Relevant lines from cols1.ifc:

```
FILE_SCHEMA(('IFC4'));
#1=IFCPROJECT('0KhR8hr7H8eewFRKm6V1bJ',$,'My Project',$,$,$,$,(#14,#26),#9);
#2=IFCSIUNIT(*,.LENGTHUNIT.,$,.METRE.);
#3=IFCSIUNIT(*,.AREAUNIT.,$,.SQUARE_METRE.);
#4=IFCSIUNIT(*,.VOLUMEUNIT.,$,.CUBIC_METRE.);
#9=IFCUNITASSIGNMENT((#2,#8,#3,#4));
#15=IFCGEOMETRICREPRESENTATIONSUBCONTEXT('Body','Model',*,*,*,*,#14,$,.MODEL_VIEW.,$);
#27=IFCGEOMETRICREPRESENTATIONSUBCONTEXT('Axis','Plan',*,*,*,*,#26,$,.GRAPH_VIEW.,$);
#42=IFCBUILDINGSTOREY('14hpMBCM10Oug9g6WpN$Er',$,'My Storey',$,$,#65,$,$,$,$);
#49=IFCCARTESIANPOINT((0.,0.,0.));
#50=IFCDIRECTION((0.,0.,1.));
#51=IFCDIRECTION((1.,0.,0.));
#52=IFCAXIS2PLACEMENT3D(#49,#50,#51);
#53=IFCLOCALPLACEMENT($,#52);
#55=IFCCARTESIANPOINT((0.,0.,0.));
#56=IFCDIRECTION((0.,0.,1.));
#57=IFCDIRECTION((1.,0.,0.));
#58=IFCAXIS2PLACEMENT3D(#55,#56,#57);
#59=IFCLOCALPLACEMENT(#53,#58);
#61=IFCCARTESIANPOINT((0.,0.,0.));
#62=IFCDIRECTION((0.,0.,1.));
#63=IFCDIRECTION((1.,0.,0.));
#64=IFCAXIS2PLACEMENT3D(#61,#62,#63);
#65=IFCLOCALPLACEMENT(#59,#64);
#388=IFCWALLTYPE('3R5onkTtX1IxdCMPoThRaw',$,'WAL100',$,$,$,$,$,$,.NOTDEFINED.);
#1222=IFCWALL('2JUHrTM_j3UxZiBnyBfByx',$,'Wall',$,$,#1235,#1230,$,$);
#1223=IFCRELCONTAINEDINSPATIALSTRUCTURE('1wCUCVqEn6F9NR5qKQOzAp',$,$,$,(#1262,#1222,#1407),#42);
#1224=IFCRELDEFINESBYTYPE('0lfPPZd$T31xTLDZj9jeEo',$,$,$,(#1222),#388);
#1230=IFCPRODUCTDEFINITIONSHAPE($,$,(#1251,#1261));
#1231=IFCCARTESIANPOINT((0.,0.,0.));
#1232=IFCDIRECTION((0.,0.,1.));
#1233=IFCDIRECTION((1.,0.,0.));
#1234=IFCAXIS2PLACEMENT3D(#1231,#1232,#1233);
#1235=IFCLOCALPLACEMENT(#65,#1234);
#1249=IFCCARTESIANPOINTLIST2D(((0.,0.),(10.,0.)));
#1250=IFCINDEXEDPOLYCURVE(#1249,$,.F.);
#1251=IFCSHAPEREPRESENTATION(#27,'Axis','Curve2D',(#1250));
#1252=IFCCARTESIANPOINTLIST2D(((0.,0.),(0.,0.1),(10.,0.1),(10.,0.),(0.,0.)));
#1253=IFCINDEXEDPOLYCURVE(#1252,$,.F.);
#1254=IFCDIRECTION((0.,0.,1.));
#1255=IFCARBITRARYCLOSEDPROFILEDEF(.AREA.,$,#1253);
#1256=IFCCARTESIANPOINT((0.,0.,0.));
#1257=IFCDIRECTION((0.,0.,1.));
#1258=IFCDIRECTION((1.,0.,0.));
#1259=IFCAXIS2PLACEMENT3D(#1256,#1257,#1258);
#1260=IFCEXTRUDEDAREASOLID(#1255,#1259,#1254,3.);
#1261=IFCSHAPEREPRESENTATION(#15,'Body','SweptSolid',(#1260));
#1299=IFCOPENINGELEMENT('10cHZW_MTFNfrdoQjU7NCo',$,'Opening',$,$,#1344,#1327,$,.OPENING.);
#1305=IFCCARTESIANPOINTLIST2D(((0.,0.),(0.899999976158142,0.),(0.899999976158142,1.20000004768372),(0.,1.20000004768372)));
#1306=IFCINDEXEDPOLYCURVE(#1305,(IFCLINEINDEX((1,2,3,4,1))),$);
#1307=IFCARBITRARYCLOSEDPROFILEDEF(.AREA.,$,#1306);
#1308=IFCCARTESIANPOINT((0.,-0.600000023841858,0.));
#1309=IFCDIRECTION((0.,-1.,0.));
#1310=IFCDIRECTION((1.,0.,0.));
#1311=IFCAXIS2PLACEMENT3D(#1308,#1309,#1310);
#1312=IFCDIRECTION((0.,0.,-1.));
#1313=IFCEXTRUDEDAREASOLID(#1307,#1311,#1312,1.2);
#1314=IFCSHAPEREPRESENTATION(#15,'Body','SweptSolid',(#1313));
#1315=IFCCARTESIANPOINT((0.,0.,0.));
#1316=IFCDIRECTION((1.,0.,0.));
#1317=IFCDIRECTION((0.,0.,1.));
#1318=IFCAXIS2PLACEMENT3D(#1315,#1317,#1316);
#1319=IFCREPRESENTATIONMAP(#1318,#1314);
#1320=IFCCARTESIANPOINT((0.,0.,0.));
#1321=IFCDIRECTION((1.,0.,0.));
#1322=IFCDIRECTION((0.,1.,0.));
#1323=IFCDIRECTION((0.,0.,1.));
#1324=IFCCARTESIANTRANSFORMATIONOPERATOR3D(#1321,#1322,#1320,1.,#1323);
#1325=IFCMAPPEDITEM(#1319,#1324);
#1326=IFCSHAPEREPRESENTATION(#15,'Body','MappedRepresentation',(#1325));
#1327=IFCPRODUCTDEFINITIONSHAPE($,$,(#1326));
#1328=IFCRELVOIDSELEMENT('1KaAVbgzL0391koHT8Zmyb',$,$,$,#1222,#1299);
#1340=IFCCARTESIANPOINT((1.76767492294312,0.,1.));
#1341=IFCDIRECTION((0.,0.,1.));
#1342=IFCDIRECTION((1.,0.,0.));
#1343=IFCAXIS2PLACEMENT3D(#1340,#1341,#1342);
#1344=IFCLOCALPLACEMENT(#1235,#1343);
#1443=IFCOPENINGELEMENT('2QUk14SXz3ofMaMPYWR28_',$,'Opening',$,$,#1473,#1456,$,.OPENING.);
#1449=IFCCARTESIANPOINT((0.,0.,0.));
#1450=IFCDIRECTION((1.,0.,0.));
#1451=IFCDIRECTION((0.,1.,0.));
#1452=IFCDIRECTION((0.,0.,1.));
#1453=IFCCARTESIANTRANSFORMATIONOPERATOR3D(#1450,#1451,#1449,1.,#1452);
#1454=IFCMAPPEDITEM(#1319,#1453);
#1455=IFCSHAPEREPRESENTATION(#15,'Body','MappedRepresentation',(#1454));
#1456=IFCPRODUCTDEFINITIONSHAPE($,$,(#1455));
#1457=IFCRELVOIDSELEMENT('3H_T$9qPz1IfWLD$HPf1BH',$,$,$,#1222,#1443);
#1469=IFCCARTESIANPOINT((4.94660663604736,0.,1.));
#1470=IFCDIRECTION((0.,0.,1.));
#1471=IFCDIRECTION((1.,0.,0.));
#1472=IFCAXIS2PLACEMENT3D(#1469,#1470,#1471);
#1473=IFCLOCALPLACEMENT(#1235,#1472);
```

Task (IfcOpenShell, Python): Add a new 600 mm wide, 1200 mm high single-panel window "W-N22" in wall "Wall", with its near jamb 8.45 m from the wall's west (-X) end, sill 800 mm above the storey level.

```python
import numpy as np
import ifcopenshell
import ifcopenshell.api.feature
import ifcopenshell.api.geometry
import ifcopenshell.api.root
import ifcopenshell.api.spatial
import ifcopenshell.geom
import ifcopenshell.util.element
import ifcopenshell.util.placement
import ifcopenshell.util.representation
import ifcopenshell.util.shape
import ifcopenshell.util.unit

model = ifcopenshell.open("cols1.ifc")
unit_scale = ifcopenshell.util.unit.calculate_unit_scale(model)
settings = ifcopenshell.geom.settings()


def volume(element):
    """Net volume in cubic metres, openings subtracted."""
    shape = ifcopenshell.geom.create_shape(settings, element)
    return ifcopenshell.util.shape.get_volume(shape.geometry)


wall = model.by_guid("2JUHrTM_j3UxZiBnyBfByx")
storey = ifcopenshell.util.element.get_container(wall, ifc_class="IfcBuildingStorey")
context = ifcopenshell.util.representation.get_context(model, "Model", "Body", "MODEL_VIEW")
before = volume(wall)

width, height, from_end, sill = 0.6, 1.2, 8.45, 0.8  # metres

# The wall runs along its own X axis, and the end named is its -X end.
wall_shape = ifcopenshell.geom.create_shape(settings, wall)
x, y, z = ifcopenshell.util.shape.get_vertices(wall_shape.geometry).T
start = x.min() + from_end
face, thickness = float(y.min()), float(y.max() - y.min())
wall_matrix = ifcopenshell.util.placement.get_local_placement(wall.ObjectPlacement)
level = ifcopenshell.util.placement.get_local_placement(storey.ObjectPlacement)[2, 3]


def in_wall(x, y):
    """Placement at x, y metres in the wall's axes, at sill height."""
    matrix = wall_matrix.copy()
    matrix[:, 3] = wall_matrix @ np.array([x / unit_scale, y / unit_scale, 0.0, 1.0])
    matrix[2, 3] = level + sill / unit_scale
    return matrix


# Opening: a box that overshoots both wall faces by 50 mm.
opening = ifcopenshell.api.root.create_entity(model, ifc_class="IfcOpeningElement", predefined_type="OPENING")
box = ifcopenshell.api.geometry.add_wall_representation(
    model, context=context, length=width, height=height, thickness=thickness + 0.1
)
ifcopenshell.api.geometry.assign_representation(model, product=opening, representation=box)
ifcopenshell.api.geometry.edit_object_placement(model, product=opening, matrix=in_wall(start, face - 0.05), is_si=False)
ifcopenshell.api.feature.add_feature(model, feature=opening, element=wall)

window = ifcopenshell.api.root.create_entity(model, ifc_class="IfcWindow", name="W-N22", predefined_type="WINDOW")
window.OverallWidth, window.OverallHeight = width / unit_scale, height / unit_scale
window.PartitioningType = "SINGLE_PANEL"
body = ifcopenshell.api.geometry.add_window_representation(
    model,
    context=context,
    overall_width=window.OverallWidth,
    overall_height=window.OverallHeight,
    partition_type="SINGLE_PANEL",
)
ifcopenshell.api.geometry.assign_representation(model, product=window, representation=body)
ifcopenshell.api.spatial.assign_container(model, products=[window], relating_structure=storey)
ifcopenshell.api.feature.add_filling(model, opening=opening, element=window)

# Centre the window in the wall's thickness.
ifcopenshell.api.geometry.edit_object_placement(model, product=window, matrix=in_wall(start, face), is_si=False)
window_shape = ifcopenshell.geom.create_shape(settings, window)
depth = ifcopenshell.util.shape.get_vertices(window_shape.geometry)[:, 1]
offset = face + thickness / 2 - (depth.min() + depth.max()) / 2
ifcopenshell.api.geometry.edit_object_placement(model, product=window, matrix=in_wall(start, offset), is_si=False)

after = volume(wall)

print(f"wall volume {before:.3f} -> {after:.3f} m3")

model.write("cols1_v2.ifc")
```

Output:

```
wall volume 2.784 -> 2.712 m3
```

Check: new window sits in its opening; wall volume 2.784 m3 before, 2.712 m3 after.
